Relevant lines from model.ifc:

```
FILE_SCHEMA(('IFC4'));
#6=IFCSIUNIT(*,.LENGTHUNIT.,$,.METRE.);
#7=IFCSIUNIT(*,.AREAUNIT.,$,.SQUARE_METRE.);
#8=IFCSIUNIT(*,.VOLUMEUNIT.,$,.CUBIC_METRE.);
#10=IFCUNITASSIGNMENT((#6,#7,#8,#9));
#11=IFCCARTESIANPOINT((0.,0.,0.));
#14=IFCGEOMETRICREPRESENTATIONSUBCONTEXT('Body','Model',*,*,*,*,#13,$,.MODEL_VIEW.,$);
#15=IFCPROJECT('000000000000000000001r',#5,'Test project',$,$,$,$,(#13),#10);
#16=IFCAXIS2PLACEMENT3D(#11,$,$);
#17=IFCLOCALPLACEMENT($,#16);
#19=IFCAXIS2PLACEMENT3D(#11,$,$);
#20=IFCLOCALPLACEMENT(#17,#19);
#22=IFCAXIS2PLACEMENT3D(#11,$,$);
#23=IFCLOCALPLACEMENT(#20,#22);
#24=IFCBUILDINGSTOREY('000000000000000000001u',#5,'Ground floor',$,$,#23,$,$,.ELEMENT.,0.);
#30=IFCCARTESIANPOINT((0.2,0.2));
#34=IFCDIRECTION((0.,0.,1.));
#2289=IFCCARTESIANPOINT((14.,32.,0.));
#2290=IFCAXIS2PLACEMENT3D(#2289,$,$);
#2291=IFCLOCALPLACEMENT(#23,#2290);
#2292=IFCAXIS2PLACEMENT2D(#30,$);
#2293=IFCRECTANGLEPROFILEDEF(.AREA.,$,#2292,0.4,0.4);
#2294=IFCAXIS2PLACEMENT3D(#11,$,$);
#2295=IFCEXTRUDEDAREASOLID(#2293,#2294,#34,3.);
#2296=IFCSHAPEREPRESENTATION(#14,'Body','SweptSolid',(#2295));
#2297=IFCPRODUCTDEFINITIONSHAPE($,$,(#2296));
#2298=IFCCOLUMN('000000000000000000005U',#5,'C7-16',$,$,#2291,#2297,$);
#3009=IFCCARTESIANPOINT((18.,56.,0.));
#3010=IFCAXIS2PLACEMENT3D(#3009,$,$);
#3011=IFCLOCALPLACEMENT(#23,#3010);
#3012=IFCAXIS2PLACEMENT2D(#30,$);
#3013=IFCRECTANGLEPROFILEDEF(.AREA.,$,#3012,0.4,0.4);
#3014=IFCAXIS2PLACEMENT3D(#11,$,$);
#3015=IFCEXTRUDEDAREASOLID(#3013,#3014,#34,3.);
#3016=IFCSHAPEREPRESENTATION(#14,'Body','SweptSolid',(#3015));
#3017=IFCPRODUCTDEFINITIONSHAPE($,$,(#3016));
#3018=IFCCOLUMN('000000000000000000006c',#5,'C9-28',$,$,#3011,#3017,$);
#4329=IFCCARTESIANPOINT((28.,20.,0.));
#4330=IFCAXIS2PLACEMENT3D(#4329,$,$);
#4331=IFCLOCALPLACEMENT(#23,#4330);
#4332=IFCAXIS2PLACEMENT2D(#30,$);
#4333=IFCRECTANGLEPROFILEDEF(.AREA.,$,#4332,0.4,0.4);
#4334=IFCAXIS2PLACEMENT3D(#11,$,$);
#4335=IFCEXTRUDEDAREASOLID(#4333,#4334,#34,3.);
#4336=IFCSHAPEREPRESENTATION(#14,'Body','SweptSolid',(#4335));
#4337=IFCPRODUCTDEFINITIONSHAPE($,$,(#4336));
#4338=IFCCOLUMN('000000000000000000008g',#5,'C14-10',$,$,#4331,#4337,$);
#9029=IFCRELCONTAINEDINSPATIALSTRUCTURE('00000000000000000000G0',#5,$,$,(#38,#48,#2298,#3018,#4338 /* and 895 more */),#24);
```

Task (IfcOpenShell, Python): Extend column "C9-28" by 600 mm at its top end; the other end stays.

```python
import ifcopenshell
import ifcopenshell.util.representation

model = ifcopenshell.open("model.ifc")

member = model.by_id(3018)
change = 0.6

# The extrusion runs towards the end named, so only its depth changes.
body = ifcopenshell.util.representation.get_representation(member, "Model", "Body")
solid = body.Items[0]
old_length = solid.Depth
solid.Depth += change

print(f"length {old_length:g} -> {solid.Depth:g}")

model.write("model_v2.ifc")
```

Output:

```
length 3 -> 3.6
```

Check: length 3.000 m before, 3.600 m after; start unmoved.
